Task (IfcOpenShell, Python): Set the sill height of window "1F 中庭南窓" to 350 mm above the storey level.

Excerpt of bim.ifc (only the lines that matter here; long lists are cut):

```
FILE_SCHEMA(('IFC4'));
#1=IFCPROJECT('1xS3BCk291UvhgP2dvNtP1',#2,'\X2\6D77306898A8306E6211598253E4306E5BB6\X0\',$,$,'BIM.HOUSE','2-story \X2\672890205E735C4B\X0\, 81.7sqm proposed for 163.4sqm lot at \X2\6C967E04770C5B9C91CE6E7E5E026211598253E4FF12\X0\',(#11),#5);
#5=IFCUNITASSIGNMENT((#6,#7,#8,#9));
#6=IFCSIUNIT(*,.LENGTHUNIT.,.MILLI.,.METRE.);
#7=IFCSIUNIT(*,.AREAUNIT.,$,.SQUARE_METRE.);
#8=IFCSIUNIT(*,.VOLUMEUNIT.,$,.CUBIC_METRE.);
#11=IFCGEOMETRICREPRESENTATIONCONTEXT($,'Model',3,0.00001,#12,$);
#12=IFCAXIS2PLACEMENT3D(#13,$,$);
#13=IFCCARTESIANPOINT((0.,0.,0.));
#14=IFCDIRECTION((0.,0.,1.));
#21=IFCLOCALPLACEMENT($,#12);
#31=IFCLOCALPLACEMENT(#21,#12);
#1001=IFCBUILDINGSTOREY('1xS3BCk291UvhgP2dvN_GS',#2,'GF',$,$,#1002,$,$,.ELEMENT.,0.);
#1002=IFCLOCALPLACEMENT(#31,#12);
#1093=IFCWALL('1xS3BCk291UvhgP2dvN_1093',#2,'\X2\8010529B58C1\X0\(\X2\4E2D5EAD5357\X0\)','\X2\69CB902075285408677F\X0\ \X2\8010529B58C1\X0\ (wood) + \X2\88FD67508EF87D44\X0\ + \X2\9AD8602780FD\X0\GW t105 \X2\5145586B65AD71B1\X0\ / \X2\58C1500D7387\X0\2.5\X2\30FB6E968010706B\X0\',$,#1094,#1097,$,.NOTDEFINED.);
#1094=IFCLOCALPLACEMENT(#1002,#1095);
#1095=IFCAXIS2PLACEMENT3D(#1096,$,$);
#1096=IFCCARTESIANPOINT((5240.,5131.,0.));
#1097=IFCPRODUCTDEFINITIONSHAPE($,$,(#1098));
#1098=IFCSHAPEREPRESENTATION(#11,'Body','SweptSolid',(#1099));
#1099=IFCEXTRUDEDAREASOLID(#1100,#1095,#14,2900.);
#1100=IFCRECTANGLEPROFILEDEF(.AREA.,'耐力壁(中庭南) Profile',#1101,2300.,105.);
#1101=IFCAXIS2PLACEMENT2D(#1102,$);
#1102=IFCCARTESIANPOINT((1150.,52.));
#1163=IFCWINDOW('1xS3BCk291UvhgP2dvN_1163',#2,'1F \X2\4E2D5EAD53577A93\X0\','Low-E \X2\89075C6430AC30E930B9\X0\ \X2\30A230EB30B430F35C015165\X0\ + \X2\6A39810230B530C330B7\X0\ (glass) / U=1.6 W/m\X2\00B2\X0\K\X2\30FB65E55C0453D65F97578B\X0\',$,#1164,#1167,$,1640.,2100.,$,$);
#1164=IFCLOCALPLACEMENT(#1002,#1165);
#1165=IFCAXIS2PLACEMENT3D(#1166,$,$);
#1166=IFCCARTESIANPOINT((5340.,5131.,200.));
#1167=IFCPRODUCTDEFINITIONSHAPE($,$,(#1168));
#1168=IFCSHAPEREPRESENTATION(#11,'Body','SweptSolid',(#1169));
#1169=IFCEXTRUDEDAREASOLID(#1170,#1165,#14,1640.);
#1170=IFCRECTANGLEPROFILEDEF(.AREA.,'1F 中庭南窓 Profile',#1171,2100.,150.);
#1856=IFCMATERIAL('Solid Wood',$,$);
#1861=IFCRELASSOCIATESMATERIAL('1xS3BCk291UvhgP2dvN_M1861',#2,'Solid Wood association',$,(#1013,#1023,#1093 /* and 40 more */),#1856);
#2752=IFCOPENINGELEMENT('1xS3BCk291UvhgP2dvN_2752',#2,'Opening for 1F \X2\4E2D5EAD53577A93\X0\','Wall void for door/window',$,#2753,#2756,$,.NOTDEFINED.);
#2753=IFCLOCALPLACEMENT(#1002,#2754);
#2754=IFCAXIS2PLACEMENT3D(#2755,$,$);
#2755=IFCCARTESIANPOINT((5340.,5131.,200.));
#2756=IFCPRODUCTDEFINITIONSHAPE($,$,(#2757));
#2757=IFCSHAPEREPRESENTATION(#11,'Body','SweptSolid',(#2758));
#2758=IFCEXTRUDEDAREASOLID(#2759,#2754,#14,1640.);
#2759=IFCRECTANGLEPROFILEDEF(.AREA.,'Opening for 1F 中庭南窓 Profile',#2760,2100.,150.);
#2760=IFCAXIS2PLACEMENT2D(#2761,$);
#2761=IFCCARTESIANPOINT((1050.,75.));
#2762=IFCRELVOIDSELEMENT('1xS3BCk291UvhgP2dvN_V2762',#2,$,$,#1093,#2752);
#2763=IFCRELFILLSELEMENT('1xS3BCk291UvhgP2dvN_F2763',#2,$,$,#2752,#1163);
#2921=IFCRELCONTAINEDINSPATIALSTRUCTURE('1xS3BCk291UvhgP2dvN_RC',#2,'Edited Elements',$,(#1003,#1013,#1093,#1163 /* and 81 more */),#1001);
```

```python
import numpy as np
import ifcopenshell
import ifcopenshell.api.geometry
import ifcopenshell.geom
import ifcopenshell.util.element
import ifcopenshell.util.placement
import ifcopenshell.util.shape
import ifcopenshell.util.unit

model = ifcopenshell.open("bim.ifc")
unit_scale = ifcopenshell.util.unit.calculate_unit_scale(model)

window = model.by_guid("1xS3BCk291UvhgP2dvN_1163")
opening = window.FillsVoids[0].RelatingOpeningElement
storey = ifcopenshell.util.element.get_container(window, ifc_class="IfcBuildingStorey")
level = ifcopenshell.util.placement.get_local_placement(storey.ObjectPlacement)[2, 3]

# The opening's origin need not be at the sill, so measure its lowest point.
shape = ifcopenshell.geom.create_shape(ifcopenshell.geom.settings(), opening)
bottom = ifcopenshell.util.shape.get_shape_bottom_elevation(shape, shape.geometry) / unit_scale
dz = level + 0.35 / unit_scale - bottom

shift = np.array([0.0, 0.0, dz])
# The window is not placed relative to its opening, so move both.
for product in (opening, window):
    matrix = ifcopenshell.util.placement.get_local_placement(product.ObjectPlacement)
    matrix[:3, 3] += shift
    ifcopenshell.api.geometry.edit_object_placement(model, product=product, matrix=matrix, is_si=False)

print(f"moved by {dz * unit_scale:+.3f} m")

model.write("bim-out.ifc")
```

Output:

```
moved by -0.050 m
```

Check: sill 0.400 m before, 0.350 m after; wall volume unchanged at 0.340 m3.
